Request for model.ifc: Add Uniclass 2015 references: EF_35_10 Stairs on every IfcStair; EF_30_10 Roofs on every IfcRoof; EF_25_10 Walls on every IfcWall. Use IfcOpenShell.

First a look at what the model holds.

```python
import ifcopenshell

model = ifcopenshell.open("model.ifc")
print(model.schema)
print("classifications:", [c.Name for c in model.by_type("IfcClassification")])
for ifc_class in ("IfcDoor", "IfcRoof", "IfcStair", "IfcWall", "IfcWindow"):
    print(ifc_class, len(model.by_type(ifc_class)))
```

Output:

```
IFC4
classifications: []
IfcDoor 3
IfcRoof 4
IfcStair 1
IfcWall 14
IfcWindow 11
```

```python
import ifcopenshell
import ifcopenshell.api.classification

model = ifcopenshell.open("model.ifc")

system = ifcopenshell.api.classification.add_classification(model, classification="Uniclass 2015")

codes = {
    "IfcStair": ("EF_35_10", "Stairs"),
    "IfcRoof": ("EF_30_10", "Roofs"),
    "IfcWall": ("EF_25_10", "Walls"),
}
for ifc_class, (code, name) in codes.items():
    products = model.by_type(ifc_class)
    ifcopenshell.api.classification.add_reference(
        model, products=products, classification=system, identification=code, name=name
    )
    print(code, len(products))

model.write("model_rev.ifc")
```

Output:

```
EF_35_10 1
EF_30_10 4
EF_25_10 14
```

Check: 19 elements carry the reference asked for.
